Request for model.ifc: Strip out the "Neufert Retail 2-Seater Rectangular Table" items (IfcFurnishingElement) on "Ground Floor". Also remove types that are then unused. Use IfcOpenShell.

First a look at what the model holds.

```python
import ifcopenshell
import ifcopenshell.util.element

model = ifcopenshell.open("model.ifc")
print(model.schema)
storey = next(s for s in model.by_type("IfcBuildingStorey") if s.Name == "Ground Floor")
furniture = [e for e in ifcopenshell.util.element.get_decomposition(storey) if e.is_a("IfcFurnishingElement")]
seen = {}
for e in furniture:
    element_type = ifcopenshell.util.element.get_type(e)
    name = element_type.Name if element_type not in (None, e) else None
    seen[name] = seen.get(name, 0) + 1
for name, count in sorted(seen.items(), key=str):
    print(count, "x", name)
```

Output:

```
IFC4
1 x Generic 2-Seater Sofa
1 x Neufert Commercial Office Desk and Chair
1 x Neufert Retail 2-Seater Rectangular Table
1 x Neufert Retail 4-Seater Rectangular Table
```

```python
import ifcopenshell
import ifcopenshell.api.root
import ifcopenshell.util.element

model = ifcopenshell.open("model.ifc")

storey = next(s for s in model.by_type("IfcBuildingStorey") if s.Name == "Ground Floor")
furniture = [e for e in ifcopenshell.util.element.get_decomposition(storey) if e.is_a("IfcFurnishingElement")]
targets = [e for e in furniture if (t := ifcopenshell.util.element.get_type(e)) not in (None, e) and t.Name == "Neufert Retail 2-Seater Rectangular Table"]
types = {ifcopenshell.util.element.get_type(e) for e in targets} - {None, *targets}

for e in targets:
    ifcopenshell.api.root.remove_product(model, product=e)
print(len(targets), "removed")

unused = [t for t in types if not ifcopenshell.util.element.get_types(t)]
for t in unused:
    ifcopenshell.api.root.remove_product(model, product=t)
print(len(unused), "unused types removed")

model.write("model_updated.ifc")
```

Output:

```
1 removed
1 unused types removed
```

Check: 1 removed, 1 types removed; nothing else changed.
